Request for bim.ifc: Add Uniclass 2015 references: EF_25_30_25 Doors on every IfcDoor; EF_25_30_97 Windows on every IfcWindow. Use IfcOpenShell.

First a look at what the model holds.

```python
import ifcopenshell

model = ifcopenshell.open("bim.ifc")
print(model.schema)
print("classifications:", [c.Name for c in model.by_type("IfcClassification")])
for ifc_class in ("IfcDoor", "IfcRoof", "IfcStair", "IfcWall", "IfcWindow"):
    print(ifc_class, len(model.by_type(ifc_class)))
```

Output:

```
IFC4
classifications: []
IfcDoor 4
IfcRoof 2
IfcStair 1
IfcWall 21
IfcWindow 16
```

```python
import ifcopenshell
import ifcopenshell.api.classification

model = ifcopenshell.open("bim.ifc")

system = ifcopenshell.api.classification.add_classification(model, classification="Uniclass 2015")

codes = {
    "IfcDoor": ("EF_25_30_25", "Doors"),
    "IfcWindow": ("EF_25_30_97", "Windows"),
}
for ifc_class, (code, name) in codes.items():
    products = model.by_type(ifc_class)
    ifcopenshell.api.classification.add_reference(
        model, products=products, classification=system, identification=code, name=name
    )
    print(code, len(products))

model.write("bim_edited.ifc")
```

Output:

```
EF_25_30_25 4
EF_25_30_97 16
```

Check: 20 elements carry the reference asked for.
